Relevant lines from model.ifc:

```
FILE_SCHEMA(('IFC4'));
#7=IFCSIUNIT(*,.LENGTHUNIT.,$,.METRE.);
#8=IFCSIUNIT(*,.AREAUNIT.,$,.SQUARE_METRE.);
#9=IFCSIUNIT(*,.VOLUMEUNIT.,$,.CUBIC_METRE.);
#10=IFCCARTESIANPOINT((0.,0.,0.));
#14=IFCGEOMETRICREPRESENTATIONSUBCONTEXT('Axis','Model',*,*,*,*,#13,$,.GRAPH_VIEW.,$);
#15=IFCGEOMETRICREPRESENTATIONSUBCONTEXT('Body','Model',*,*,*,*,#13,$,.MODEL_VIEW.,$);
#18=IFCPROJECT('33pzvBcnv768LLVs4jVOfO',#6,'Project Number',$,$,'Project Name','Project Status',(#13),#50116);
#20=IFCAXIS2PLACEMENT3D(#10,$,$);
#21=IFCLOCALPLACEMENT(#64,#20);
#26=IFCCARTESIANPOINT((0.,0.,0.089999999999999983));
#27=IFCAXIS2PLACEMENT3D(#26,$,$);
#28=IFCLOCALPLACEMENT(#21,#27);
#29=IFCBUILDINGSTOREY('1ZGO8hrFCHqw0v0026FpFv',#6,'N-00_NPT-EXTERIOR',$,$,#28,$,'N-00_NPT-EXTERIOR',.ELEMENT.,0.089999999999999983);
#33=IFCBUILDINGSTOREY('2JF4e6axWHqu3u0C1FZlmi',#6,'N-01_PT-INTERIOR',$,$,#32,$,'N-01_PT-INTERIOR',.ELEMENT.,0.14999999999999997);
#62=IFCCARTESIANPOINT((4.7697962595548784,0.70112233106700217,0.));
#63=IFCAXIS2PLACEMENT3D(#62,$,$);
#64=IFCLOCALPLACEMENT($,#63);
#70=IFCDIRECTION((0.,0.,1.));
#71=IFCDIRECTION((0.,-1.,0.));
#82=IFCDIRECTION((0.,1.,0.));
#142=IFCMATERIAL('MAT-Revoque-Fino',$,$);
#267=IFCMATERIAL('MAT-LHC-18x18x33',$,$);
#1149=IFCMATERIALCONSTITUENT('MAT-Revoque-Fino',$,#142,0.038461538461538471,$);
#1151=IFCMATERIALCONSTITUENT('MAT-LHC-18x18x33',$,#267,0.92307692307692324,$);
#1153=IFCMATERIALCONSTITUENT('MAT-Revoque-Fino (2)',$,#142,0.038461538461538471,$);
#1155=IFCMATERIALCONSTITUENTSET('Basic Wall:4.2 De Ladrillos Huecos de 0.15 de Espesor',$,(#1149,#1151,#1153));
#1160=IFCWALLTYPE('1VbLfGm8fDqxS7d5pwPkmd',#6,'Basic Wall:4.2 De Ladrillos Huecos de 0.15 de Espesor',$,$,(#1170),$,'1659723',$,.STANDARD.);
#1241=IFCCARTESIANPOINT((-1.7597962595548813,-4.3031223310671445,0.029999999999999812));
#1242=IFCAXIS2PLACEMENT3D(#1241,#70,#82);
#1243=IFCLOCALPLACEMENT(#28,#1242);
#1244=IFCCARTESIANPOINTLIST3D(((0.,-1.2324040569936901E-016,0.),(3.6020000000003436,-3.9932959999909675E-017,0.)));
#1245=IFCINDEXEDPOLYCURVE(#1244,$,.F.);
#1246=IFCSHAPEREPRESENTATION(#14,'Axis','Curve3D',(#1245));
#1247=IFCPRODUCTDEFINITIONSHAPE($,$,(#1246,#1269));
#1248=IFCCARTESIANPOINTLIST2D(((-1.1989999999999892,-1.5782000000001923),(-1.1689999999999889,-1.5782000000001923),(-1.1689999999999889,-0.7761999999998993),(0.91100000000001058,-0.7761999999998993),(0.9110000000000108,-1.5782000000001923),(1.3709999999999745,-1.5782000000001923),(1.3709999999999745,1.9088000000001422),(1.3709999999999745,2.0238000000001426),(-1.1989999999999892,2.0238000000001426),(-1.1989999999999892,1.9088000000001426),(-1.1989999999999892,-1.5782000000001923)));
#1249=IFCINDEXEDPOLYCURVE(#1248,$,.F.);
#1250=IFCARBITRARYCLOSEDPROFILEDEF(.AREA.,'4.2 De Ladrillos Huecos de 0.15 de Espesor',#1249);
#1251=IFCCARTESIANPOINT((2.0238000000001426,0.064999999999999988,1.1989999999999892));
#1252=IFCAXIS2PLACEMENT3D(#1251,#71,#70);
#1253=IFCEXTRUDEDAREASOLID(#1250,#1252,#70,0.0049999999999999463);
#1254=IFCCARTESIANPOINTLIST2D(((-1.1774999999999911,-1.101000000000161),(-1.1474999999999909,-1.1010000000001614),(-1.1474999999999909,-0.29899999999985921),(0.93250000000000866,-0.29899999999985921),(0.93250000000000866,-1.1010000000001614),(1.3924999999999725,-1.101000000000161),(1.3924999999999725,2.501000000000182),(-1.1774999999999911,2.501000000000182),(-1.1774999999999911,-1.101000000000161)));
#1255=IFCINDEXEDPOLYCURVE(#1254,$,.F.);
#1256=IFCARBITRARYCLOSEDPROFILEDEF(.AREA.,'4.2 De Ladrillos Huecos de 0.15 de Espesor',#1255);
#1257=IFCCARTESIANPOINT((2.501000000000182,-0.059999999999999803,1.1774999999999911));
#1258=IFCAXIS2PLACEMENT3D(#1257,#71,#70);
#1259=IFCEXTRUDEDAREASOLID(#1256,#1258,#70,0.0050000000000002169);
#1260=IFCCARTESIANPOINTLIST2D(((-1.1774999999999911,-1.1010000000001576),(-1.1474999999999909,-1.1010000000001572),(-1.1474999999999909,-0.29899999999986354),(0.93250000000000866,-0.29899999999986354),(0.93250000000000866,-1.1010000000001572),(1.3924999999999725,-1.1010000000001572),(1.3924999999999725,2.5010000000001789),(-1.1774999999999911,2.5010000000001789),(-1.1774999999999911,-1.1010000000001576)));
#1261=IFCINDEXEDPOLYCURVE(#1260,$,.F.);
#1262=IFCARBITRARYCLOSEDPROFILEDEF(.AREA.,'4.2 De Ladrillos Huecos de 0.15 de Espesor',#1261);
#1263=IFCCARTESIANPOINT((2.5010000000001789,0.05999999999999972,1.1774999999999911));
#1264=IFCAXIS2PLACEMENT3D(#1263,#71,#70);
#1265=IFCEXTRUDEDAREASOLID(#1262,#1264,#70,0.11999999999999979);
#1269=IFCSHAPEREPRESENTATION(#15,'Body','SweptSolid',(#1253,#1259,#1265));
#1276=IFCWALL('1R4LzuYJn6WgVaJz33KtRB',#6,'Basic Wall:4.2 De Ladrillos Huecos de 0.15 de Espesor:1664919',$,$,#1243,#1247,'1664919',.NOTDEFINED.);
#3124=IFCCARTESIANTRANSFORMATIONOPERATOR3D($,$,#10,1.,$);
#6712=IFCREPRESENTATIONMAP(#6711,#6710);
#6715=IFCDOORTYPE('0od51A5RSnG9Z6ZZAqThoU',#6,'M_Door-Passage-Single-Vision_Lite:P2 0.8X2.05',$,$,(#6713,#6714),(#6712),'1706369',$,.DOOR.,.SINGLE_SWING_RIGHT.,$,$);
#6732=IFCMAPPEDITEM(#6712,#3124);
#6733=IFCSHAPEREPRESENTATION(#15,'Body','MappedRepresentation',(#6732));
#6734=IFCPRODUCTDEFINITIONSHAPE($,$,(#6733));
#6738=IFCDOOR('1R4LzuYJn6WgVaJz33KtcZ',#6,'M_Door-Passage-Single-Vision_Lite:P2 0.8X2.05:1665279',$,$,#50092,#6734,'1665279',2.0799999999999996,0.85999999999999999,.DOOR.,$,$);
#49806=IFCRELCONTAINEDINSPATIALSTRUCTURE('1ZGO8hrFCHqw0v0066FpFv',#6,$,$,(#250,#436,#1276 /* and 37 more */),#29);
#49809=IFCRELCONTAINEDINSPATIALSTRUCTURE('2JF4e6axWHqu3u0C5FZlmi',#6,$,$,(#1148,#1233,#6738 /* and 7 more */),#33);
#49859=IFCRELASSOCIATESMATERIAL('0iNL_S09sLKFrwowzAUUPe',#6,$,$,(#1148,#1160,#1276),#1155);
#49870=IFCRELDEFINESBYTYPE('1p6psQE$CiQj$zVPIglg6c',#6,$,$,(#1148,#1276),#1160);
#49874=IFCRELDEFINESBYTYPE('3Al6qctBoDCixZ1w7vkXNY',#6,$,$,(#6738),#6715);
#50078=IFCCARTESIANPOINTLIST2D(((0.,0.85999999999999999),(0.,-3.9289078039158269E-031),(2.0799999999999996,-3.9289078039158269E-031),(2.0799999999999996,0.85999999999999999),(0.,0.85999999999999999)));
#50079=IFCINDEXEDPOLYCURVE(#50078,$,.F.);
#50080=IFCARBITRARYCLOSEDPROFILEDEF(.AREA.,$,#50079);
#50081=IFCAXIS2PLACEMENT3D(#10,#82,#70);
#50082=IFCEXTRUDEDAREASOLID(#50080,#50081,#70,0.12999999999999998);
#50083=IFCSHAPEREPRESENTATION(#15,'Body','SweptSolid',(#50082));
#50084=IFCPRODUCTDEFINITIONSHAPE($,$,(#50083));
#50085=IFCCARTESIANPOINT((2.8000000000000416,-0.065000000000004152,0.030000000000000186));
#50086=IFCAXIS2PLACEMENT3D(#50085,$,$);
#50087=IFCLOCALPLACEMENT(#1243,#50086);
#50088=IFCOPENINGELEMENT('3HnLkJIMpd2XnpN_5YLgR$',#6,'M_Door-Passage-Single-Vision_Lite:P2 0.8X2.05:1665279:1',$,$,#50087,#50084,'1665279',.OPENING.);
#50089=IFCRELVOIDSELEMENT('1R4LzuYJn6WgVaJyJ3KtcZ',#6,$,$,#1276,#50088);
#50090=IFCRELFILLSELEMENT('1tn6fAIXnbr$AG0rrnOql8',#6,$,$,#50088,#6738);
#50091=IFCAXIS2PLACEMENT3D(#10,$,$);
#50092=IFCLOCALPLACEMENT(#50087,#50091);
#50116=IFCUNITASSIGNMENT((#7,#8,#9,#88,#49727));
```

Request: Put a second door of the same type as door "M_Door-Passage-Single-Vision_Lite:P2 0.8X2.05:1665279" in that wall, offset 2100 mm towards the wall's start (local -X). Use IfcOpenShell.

```python
import ifcopenshell
import ifcopenshell.api.feature
import ifcopenshell.api.geometry
import ifcopenshell.api.root
import ifcopenshell.geom
import ifcopenshell.util.element
import ifcopenshell.util.placement
import ifcopenshell.util.shape
import ifcopenshell.util.unit

model = ifcopenshell.open("model.ifc")
unit_scale = ifcopenshell.util.unit.calculate_unit_scale(model)
settings = ifcopenshell.geom.settings()


def volume(element):
    """Net volume in cubic metres, openings subtracted."""
    shape = ifcopenshell.geom.create_shape(settings, element)
    return ifcopenshell.util.shape.get_volume(shape.geometry)


def reuse_history(source, copy):
    """copy_class also copies each property set's owner history, people and application; keep the originals."""
    for rel in copy.IsDefinedBy:
        if rel.is_a("IfcRelDefinesByProperties") and (history := rel.RelatingPropertyDefinition.OwnerHistory):
            rel.RelatingPropertyDefinition.OwnerHistory = source.OwnerHistory
            ifcopenshell.util.element.remove_deep2(model, history)


door = model.by_guid("1R4LzuYJn6WgVaJz33KtcZ")
opening = door.FillsVoids[0].RelatingOpeningElement
wall = opening.VoidsElements[0].RelatingBuildingElement
before = volume(wall)
shift = ifcopenshell.util.placement.get_local_placement(wall.ObjectPlacement)[:3, 0] * -2.1 / unit_scale

# copy_class copies the void relationship, type, container and properties, but no geometry.
new_opening = ifcopenshell.api.root.copy_class(model, product=opening)
new_opening.Representation = ifcopenshell.util.element.copy_deep(
    model, opening.Representation, exclude=["IfcGeometricRepresentationContext", "IfcRepresentationMap"]
)
new_opening.Name = "M_Door-Passage-Single-Vision_Lite:P2 0.8X2.05"
new_opening.Tag = None
new_door = ifcopenshell.api.root.copy_class(model, product=door)
new_door.Representation = ifcopenshell.util.element.copy_deep(
    model, door.Representation, exclude=["IfcGeometricRepresentationContext", "IfcRepresentationMap"]
)
new_door.Name = "M_Door-Passage-Single-Vision_Lite:P2 0.8X2.05"
new_door.Tag = None
reuse_history(door, new_door)
ifcopenshell.api.feature.add_filling(model, opening=new_opening, element=new_door)

for old, new in ((opening, new_opening), (door, new_door)):
    matrix = ifcopenshell.util.placement.get_local_placement(old.ObjectPlacement)
    matrix[:3, 3] += shift
    ifcopenshell.api.geometry.edit_object_placement(model, product=new, matrix=matrix, is_si=False)

after = volume(wall)

print(f"wall volume {before:.3f} -> {after:.3f} m3")

model.write("model_v2.ifc")
```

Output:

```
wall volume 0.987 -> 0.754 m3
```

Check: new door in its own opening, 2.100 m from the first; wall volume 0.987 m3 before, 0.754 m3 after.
